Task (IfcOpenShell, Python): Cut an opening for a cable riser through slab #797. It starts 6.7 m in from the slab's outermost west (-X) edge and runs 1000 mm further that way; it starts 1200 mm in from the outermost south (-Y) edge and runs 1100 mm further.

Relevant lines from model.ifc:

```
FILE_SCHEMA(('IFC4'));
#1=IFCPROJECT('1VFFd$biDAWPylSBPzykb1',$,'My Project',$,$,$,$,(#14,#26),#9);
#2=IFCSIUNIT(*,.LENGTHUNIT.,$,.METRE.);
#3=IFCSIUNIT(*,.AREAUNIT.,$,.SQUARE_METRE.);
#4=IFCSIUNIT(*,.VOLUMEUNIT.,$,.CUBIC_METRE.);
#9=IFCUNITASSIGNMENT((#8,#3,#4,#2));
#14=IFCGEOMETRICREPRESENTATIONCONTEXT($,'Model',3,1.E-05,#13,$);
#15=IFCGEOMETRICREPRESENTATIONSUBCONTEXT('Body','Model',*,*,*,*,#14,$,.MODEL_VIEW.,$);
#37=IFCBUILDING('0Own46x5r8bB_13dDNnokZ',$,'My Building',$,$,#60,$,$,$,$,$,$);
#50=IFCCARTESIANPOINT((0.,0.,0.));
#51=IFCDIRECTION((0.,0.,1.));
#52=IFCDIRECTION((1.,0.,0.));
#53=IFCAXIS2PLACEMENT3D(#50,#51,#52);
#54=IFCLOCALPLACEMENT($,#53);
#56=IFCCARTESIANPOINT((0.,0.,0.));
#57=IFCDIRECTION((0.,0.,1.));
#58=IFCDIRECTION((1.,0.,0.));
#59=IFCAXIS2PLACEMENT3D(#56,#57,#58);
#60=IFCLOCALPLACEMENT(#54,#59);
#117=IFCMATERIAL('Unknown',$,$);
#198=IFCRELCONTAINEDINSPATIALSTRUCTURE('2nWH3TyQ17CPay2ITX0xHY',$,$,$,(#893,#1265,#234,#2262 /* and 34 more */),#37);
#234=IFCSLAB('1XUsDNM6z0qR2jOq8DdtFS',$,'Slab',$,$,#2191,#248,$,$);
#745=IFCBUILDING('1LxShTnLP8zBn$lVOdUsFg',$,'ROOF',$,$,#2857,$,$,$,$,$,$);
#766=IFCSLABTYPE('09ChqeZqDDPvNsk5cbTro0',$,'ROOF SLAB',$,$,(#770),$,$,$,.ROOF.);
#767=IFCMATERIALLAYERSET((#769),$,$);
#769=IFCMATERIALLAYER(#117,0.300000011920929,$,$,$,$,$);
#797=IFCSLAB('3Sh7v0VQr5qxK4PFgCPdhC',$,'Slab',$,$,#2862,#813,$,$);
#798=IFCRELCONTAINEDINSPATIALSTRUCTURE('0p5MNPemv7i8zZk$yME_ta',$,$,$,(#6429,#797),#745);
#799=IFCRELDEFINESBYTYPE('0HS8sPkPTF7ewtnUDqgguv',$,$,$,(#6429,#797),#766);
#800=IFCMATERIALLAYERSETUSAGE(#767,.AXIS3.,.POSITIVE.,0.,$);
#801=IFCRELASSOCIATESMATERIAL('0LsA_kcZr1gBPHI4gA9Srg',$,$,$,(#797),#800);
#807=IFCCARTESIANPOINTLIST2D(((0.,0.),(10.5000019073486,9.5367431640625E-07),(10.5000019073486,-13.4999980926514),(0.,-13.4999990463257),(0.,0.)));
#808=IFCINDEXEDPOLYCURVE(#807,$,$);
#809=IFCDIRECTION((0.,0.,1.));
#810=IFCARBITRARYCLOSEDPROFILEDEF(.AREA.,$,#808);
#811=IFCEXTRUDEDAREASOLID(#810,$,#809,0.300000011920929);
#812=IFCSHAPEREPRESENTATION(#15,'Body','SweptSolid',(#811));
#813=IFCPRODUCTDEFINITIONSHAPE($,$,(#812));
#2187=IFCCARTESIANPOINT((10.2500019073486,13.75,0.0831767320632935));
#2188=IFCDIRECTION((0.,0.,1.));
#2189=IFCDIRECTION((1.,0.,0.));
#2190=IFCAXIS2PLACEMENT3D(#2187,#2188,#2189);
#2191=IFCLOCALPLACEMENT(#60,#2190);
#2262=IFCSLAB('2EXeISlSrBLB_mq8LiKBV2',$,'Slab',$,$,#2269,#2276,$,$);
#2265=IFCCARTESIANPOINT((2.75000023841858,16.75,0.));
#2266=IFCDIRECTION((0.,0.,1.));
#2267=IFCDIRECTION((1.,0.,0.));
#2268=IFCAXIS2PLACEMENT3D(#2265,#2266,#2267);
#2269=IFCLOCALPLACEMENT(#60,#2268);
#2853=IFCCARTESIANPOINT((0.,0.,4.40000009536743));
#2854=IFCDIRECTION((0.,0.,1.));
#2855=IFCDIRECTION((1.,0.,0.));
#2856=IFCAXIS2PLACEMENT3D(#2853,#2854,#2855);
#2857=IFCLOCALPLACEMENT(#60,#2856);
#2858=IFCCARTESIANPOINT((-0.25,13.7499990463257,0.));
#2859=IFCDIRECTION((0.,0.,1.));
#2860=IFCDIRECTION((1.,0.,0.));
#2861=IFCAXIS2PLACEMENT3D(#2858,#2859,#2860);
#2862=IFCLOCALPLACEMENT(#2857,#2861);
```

```python
import numpy as np
import ifcopenshell
import ifcopenshell.api.feature
import ifcopenshell.api.geometry
import ifcopenshell.api.root
import ifcopenshell.geom
import ifcopenshell.util.placement
import ifcopenshell.util.representation
import ifcopenshell.util.shape
import ifcopenshell.util.unit

model = ifcopenshell.open("model.ifc")
unit_scale = ifcopenshell.util.unit.calculate_unit_scale(model)
settings = ifcopenshell.geom.settings()


def volume(element):
    """Net volume in cubic metres, openings subtracted."""
    shape = ifcopenshell.geom.create_shape(settings, element)
    return ifcopenshell.util.shape.get_volume(shape.geometry)


slab = model.by_id(797)
before = volume(slab)

# Extent in the slab's own axes, in metres. The edges named are its -X and -Y sides.
slab_shape = ifcopenshell.geom.create_shape(settings, slab)
vertices = ifcopenshell.util.shape.get_vertices(slab_shape.geometry)
x_min, y_min, bottom = vertices.min(axis=0)
top = vertices[:, 2].max()

opening = ifcopenshell.api.root.create_entity(model, ifc_class="IfcOpeningElement", name="Cable riser opening", predefined_type="OPENING")
context = ifcopenshell.util.representation.get_context(model, "Model", "Body", "MODEL_VIEW")
width, depth = 1, 1.1
outline = [(0.0, 0.0), (width, 0.0), (width, depth), (0.0, depth), (0.0, 0.0)]
# Overshoot both faces by 50 mm so the cut is clean.
shape = ifcopenshell.api.geometry.add_slab_representation(
    model, context=context, depth=top - bottom + 0.1, polyline=outline
)
ifcopenshell.api.geometry.assign_representation(model, product=opening, representation=shape)

matrix = ifcopenshell.util.placement.get_local_placement(slab.ObjectPlacement)
matrix[:, 3] = matrix @ np.append(np.array([x_min + 6.7, y_min + 1.2, bottom - 0.05]) / unit_scale, 1.0)
ifcopenshell.api.geometry.edit_object_placement(model, product=opening, matrix=matrix, is_si=False)
ifcopenshell.api.feature.add_feature(model, feature=opening, element=slab)

after = volume(slab)

print(f"slab volume {before:.3f} -> {after:.3f} m3")

model.write("model_updated.ifc")
```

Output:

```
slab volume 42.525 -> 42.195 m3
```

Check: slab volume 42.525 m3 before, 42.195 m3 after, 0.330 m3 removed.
